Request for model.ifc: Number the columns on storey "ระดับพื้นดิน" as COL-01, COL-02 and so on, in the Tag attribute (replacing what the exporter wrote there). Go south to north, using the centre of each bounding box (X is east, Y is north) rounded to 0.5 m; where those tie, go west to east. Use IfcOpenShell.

First a look at what the model holds.

```python
import ifcopenshell
import ifcopenshell.util.element
import ifcopenshell.util.placement

model = ifcopenshell.open("model.ifc")
print(model.schema)
storey = next(s for s in model.by_type("IfcBuildingStorey") if s.Name == "ระดับพื้นดิน")
columns = [e for e in ifcopenshell.util.element.get_decomposition(storey) if e.is_a("IfcColumn")]
for e in sorted(columns, key=lambda e: e.id()):
    origin = ifcopenshell.util.placement.get_local_placement(e.ObjectPlacement)[:3, 3]
    print(e.id(), e.Tag, e.Name, origin.round(2) + 0.0, sep=" | ")
```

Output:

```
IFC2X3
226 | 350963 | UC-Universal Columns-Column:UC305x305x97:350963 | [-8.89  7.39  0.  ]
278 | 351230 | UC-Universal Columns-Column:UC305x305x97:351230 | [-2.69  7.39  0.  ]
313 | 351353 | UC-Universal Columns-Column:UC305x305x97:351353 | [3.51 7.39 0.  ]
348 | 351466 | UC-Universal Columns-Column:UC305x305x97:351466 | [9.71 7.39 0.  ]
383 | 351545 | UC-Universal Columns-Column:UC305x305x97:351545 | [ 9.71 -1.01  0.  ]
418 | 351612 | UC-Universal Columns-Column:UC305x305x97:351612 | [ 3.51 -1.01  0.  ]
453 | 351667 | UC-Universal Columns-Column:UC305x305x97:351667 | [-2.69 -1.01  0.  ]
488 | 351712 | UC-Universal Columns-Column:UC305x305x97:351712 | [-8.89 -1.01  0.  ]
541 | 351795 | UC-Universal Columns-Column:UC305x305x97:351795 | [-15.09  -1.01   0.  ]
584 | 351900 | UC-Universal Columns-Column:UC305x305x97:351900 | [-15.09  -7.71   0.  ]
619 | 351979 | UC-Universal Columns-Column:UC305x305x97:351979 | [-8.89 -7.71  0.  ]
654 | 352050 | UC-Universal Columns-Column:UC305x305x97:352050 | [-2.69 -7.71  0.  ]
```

```python
import ifcopenshell
import ifcopenshell.geom
import ifcopenshell.util.element
import ifcopenshell.util.shape

model = ifcopenshell.open("model.ifc")
settings = ifcopenshell.geom.settings()
settings.set("use-world-coords", True)


def centre(element):
    shape = ifcopenshell.geom.create_shape(settings, element)
    return ifcopenshell.util.shape.get_bbox_centroid(shape.geometry)


storey = next(s for s in model.by_type("IfcBuildingStorey") if s.Name == "ระดับพื้นดิน")
columns = [e for e in ifcopenshell.util.element.get_decomposition(storey) if e.is_a("IfcColumn")]

# Insertion points can sit at a corner or the storey origin, so sort by the geometry (in metres).
centres = {e: centre(e) for e in columns}
columns.sort(key=lambda e: (round(centres[e][1] / 0.5), centres[e][0]))

for i, e in enumerate(columns, start=1):
    number = f"COL-{i:02d}"
    e.Tag = number
    print(e.id(), number)

model.write("model_v2.ifc")
```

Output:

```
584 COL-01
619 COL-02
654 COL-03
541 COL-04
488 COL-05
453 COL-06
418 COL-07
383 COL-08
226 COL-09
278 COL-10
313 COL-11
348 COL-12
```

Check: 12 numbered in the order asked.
